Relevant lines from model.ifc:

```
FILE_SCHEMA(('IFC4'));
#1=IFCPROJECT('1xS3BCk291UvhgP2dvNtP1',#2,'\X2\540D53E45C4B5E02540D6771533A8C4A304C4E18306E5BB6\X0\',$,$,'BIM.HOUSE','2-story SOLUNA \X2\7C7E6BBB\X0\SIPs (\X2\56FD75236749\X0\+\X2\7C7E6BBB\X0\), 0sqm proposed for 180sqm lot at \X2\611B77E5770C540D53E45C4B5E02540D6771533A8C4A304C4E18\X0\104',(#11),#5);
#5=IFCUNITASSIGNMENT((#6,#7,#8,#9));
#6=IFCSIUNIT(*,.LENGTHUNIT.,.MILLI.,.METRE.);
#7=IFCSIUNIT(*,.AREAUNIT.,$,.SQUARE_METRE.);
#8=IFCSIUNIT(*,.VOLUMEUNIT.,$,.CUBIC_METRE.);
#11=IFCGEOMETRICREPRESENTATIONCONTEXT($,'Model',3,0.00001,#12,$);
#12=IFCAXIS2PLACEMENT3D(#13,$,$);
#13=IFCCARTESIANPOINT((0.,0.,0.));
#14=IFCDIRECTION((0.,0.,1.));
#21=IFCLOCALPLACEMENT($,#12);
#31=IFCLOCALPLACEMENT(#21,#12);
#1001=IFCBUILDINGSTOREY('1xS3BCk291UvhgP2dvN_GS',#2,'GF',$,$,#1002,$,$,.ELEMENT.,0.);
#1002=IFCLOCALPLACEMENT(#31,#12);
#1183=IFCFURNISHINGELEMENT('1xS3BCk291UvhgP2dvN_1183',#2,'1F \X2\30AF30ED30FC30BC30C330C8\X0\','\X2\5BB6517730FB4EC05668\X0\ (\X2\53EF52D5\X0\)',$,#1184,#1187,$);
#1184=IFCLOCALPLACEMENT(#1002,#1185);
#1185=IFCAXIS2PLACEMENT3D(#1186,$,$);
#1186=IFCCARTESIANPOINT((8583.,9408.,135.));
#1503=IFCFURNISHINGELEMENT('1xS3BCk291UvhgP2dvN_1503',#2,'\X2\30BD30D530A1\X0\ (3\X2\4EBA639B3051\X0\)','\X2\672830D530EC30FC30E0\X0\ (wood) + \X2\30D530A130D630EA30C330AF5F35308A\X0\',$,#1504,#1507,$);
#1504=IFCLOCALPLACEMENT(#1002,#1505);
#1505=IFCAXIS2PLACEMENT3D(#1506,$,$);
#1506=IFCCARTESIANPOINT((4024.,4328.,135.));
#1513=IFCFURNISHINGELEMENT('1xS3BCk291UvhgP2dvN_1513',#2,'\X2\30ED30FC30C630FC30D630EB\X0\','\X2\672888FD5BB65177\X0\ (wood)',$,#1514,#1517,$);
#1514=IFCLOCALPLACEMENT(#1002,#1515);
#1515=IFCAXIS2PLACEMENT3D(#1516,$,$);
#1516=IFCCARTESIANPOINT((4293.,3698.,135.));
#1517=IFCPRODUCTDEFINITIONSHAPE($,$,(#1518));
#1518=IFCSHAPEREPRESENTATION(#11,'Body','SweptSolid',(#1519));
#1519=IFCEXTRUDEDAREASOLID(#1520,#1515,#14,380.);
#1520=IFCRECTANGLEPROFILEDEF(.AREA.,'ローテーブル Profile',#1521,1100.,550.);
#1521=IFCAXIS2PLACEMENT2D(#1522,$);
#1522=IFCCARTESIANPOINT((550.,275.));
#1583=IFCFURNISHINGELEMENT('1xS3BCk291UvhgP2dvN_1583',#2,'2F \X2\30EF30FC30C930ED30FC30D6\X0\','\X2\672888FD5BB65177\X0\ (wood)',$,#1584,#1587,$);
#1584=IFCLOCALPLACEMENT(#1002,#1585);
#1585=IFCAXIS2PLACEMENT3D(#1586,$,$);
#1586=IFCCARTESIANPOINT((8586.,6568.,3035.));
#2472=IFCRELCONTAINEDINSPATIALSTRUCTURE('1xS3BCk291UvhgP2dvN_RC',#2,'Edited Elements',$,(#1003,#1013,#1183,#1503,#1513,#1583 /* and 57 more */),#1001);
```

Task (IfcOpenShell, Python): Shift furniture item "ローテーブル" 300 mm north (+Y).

```python
import ifcopenshell
import ifcopenshell.api.geometry
import ifcopenshell.util.placement
import ifcopenshell.util.unit

model = ifcopenshell.open("model.ifc")
unit_scale = ifcopenshell.util.unit.calculate_unit_scale(model)

item = model.by_guid("1xS3BCk291UvhgP2dvN_1513")
matrix = ifcopenshell.util.placement.get_local_placement(item.ObjectPlacement)
matrix[1, 3] += 0.3 / unit_scale
ifcopenshell.api.geometry.edit_object_placement(model, product=item, matrix=matrix, is_si=False)

print(ifcopenshell.util.placement.get_local_placement(item.ObjectPlacement).round(3) + 0.0)

model.write("model-out.ifc")
```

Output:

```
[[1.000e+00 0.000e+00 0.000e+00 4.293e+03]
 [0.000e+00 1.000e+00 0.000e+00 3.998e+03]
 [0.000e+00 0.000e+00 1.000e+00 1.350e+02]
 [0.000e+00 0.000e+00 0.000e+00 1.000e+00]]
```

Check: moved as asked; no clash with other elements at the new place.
